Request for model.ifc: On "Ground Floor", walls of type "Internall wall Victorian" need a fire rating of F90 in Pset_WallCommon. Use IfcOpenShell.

First a look at what the model holds.

```python
import ifcopenshell
import ifcopenshell.util.element

model = ifcopenshell.open("model.ifc")
print(model.schema)
storey = next(s for s in model.by_type("IfcBuildingStorey") if s.Name == "Ground Floor")
walls = [e for e in ifcopenshell.util.element.get_decomposition(storey) if e.is_a("IfcWall")]
seen = {}
for e in walls:
    element_type = ifcopenshell.util.element.get_type(e)
    key = (element_type.Name if element_type != e and element_type else None, ifcopenshell.util.element.get_pset(e, "Pset_WallCommon", "FireRating"))
    seen[key] = seen.get(key, 0) + 1
for (name, value), count in sorted(seen.items(), key=str):
    print(count, "x", name, "|", value)
```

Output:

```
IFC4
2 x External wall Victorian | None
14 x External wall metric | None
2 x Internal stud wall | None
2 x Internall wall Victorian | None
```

```python
import ifcopenshell
import ifcopenshell.api.pset
import ifcopenshell.util.element

model = ifcopenshell.open("model.ifc")

storey = next(s for s in model.by_type("IfcBuildingStorey") if s.Name == "Ground Floor")
walls = [e for e in ifcopenshell.util.element.get_decomposition(storey) if e.is_a("IfcWall")]

count = 0
for e in walls:
    element_type = ifcopenshell.util.element.get_type(e)
    if element_type in (None, e) or element_type.Name != "Internall wall Victorian":
        continue
    # add_pset returns the element's existing set when there is one.
    pset = ifcopenshell.api.pset.add_pset(model, product=e, name="Pset_WallCommon")
    ifcopenshell.api.pset.edit_pset(model, pset=pset, properties={"FireRating": "F90"})
    count += 1

print(count, "walls updated")

model.write("model_edited.ifc")
```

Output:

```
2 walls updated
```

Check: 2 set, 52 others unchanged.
